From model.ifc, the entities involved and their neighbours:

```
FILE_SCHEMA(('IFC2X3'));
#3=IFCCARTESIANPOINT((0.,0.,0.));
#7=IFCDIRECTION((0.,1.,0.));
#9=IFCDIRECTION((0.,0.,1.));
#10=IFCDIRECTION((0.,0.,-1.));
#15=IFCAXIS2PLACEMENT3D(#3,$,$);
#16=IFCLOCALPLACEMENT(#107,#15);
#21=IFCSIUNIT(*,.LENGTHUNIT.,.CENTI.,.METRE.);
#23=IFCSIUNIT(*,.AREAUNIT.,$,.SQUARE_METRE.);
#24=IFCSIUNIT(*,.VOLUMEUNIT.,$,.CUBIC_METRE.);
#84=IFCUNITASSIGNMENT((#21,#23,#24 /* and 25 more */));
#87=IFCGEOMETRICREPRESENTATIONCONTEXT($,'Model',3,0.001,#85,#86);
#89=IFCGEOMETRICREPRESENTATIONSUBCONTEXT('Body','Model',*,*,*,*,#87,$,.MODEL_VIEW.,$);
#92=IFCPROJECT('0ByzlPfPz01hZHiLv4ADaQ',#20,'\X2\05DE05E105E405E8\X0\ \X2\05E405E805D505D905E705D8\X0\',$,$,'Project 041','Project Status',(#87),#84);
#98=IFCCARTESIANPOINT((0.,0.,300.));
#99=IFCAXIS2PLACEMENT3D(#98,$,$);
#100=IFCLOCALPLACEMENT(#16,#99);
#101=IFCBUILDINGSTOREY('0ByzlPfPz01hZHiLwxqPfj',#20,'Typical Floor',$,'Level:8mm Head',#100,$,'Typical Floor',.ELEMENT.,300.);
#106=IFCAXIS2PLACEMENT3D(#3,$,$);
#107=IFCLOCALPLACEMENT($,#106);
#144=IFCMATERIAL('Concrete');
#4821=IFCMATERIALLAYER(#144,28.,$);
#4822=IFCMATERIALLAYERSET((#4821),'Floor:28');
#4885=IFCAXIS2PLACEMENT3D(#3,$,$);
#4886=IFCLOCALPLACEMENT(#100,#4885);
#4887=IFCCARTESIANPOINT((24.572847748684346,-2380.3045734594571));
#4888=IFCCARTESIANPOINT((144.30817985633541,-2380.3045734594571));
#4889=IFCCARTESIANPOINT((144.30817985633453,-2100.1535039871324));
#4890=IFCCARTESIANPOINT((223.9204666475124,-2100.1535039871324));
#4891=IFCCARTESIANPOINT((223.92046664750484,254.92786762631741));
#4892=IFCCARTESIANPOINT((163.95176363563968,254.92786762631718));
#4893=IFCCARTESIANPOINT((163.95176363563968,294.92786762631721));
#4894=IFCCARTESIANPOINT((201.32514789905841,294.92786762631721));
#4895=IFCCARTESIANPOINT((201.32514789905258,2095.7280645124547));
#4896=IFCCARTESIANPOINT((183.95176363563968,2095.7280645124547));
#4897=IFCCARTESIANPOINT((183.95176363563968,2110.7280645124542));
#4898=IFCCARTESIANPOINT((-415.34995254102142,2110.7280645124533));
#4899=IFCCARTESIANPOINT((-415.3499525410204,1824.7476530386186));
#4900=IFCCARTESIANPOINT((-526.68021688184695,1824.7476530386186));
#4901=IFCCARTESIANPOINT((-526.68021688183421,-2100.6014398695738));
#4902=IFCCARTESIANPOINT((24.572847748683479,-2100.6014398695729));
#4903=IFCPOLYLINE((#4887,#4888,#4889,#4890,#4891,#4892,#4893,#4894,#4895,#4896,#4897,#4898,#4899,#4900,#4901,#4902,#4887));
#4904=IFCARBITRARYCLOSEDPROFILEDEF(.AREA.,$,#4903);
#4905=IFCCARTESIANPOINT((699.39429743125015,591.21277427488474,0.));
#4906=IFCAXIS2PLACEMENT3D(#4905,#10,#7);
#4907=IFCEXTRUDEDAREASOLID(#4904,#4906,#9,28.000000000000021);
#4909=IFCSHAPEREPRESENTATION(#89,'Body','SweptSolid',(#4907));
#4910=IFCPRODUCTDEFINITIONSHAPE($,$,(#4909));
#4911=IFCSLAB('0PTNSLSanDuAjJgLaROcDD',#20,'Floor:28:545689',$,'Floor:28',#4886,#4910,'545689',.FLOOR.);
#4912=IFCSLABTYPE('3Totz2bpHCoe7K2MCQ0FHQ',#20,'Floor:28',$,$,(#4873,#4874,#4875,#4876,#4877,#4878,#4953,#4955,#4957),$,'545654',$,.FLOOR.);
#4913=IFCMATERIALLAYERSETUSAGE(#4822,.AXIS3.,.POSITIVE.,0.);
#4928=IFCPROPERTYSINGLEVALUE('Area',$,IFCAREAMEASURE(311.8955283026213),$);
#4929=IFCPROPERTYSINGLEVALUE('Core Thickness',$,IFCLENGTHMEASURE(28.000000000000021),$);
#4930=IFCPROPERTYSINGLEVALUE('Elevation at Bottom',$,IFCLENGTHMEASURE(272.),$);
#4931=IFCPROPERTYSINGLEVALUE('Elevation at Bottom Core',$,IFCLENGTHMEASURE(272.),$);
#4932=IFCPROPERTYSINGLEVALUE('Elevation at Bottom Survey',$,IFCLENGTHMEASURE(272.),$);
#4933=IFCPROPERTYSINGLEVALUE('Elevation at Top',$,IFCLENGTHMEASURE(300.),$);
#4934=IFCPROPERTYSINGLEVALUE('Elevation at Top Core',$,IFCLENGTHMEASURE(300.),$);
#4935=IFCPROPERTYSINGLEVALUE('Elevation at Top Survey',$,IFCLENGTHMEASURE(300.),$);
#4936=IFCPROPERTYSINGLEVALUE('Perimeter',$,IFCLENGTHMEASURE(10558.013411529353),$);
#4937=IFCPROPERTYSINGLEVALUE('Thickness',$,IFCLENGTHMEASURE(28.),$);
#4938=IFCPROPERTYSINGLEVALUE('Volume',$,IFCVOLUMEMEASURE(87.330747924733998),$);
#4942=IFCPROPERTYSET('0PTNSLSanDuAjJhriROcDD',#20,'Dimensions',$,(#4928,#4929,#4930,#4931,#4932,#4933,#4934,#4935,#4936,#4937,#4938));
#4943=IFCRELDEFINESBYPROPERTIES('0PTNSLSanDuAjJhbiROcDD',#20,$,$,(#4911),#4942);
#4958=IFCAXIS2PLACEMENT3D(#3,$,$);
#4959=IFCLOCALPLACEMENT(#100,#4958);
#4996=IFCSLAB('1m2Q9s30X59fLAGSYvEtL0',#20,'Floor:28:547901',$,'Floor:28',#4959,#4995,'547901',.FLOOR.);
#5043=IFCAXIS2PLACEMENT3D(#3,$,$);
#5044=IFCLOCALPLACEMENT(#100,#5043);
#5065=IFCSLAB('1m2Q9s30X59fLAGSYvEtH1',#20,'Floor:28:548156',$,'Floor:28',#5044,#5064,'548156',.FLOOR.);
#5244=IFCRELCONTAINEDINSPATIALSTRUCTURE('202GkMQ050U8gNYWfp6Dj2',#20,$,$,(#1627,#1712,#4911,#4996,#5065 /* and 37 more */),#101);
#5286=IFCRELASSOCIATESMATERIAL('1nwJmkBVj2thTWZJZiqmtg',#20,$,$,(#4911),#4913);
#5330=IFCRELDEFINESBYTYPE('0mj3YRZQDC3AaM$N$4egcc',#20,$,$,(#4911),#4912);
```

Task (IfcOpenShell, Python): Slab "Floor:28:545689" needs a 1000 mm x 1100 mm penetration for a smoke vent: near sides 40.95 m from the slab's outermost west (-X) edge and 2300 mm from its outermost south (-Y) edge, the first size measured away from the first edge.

```python
import numpy as np
import ifcopenshell
import ifcopenshell.api.feature
import ifcopenshell.api.geometry
import ifcopenshell.api.pset
import ifcopenshell.api.root
import ifcopenshell.geom
import ifcopenshell.util.element
import ifcopenshell.util.placement
import ifcopenshell.util.representation
import ifcopenshell.util.shape
import ifcopenshell.util.unit

model = ifcopenshell.open("model.ifc")
unit_scale = ifcopenshell.util.unit.calculate_unit_scale(model)
area_scale = ifcopenshell.util.unit.calculate_unit_scale(model, "AREAUNIT")
volume_scale = ifcopenshell.util.unit.calculate_unit_scale(model, "VOLUMEUNIT")
settings = ifcopenshell.geom.settings()


def volume(element):
    """Net volume in cubic metres, openings subtracted."""
    shape = ifcopenshell.geom.create_shape(settings, element)
    return ifcopenshell.util.shape.get_volume(shape.geometry)


slab = model.by_guid("0PTNSLSanDuAjJgLaROcDD")
before = volume(slab)

# Extent in the slab's own axes, in metres. The edges named are its -X and -Y sides.
slab_shape = ifcopenshell.geom.create_shape(settings, slab)
vertices = ifcopenshell.util.shape.get_vertices(slab_shape.geometry)
x_min, y_min, bottom = vertices.min(axis=0)
top = vertices[:, 2].max()

opening = ifcopenshell.api.root.create_entity(model, ifc_class="IfcOpeningElement", name="Smoke vent opening")
context = ifcopenshell.util.representation.get_context(model, "Model", "Body", "MODEL_VIEW")
width, depth = 1, 1.1
outline = [(0.0, 0.0), (width, 0.0), (width, depth), (0.0, depth), (0.0, 0.0)]
# Overshoot both faces by 50 mm so the cut is clean.
shape = ifcopenshell.api.geometry.add_slab_representation(
    model, context=context, depth=top - bottom + 0.1, polyline=outline
)
ifcopenshell.api.geometry.assign_representation(model, product=opening, representation=shape)

matrix = ifcopenshell.util.placement.get_local_placement(slab.ObjectPlacement)
matrix[:, 3] = matrix @ np.append(np.array([x_min + 40.95, y_min + 2.3, bottom - 0.05]) / unit_scale, 1.0)
ifcopenshell.api.geometry.edit_object_placement(model, product=opening, matrix=matrix, is_si=False)
ifcopenshell.api.feature.add_feature(model, feature=opening, element=slab)

after = volume(slab)

# Update the slab's stored quantities.
pset = model.by_id(ifcopenshell.util.element.get_pset(slab, "Dimensions", should_inherit=False)["id"])
ifcopenshell.api.pset.edit_pset(model, pset=pset, properties={
    "Area": model.create_entity("IfcAreaMeasure", after / (top - bottom) / area_scale),
    "Volume": model.create_entity("IfcVolumeMeasure", after / volume_scale),
})

print(f"slab volume {before:.3f} -> {after:.3f} m3")

model.write("model_edited.ifc")
```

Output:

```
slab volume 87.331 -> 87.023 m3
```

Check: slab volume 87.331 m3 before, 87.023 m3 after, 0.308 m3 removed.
